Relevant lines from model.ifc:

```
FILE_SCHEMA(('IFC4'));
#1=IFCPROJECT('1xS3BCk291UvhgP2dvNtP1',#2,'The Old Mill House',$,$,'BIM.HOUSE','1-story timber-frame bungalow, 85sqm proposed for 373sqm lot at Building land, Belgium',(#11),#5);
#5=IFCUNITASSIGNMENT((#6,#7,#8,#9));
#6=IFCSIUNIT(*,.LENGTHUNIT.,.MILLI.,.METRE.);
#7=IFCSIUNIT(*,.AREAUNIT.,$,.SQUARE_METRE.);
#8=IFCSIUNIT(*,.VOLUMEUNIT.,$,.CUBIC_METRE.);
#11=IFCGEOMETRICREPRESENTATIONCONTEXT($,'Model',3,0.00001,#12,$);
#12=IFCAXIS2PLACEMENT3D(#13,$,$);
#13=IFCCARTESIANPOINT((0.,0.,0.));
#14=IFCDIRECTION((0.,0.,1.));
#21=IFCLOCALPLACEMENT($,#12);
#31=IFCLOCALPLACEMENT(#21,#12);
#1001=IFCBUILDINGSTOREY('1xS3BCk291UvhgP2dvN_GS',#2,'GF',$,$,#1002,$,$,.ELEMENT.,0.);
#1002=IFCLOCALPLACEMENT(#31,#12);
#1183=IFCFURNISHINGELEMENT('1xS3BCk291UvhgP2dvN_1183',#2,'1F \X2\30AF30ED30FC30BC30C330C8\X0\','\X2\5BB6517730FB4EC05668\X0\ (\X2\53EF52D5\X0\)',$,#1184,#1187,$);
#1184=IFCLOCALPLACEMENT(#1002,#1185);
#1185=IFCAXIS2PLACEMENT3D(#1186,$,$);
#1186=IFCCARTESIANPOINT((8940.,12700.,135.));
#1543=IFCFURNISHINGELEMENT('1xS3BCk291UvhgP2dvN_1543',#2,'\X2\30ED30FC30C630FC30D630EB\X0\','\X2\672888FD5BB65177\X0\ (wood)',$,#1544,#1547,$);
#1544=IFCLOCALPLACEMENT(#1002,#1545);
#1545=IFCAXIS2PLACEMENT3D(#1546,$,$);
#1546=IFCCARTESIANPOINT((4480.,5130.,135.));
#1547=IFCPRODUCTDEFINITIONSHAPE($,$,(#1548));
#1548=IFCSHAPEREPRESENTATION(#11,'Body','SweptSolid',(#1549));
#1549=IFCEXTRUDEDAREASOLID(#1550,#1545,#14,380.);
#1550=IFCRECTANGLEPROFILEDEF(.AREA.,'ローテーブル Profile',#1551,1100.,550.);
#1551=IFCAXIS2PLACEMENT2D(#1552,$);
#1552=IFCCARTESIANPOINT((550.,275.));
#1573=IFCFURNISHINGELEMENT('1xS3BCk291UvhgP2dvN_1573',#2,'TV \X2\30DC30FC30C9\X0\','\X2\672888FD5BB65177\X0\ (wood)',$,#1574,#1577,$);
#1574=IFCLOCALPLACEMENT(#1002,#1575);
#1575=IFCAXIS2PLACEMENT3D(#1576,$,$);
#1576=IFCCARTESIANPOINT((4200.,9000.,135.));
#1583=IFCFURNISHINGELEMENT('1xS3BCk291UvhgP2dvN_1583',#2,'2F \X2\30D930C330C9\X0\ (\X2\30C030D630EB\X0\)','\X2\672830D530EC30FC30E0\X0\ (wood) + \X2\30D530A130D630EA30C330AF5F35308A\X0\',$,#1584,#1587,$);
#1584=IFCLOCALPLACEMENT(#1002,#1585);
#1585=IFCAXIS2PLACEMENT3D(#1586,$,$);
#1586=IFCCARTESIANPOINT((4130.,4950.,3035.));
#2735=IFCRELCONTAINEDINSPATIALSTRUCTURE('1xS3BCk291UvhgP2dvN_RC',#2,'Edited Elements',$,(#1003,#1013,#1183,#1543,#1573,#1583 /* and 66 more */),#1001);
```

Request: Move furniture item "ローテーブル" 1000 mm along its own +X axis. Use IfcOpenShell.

```python
import ifcopenshell
import ifcopenshell.api.geometry
import ifcopenshell.util.placement

model = ifcopenshell.open("model.ifc")

item = model.by_id(1543)
matrix = ifcopenshell.util.placement.get_local_placement(item.ObjectPlacement)
matrix[:3, 3] += matrix[:3, 0] * 1000.0
ifcopenshell.api.geometry.edit_object_placement(model, product=item, matrix=matrix, is_si=False)

print(ifcopenshell.util.placement.get_local_placement(item.ObjectPlacement).round(3) + 0.0)

model.write("model_updated.ifc")
```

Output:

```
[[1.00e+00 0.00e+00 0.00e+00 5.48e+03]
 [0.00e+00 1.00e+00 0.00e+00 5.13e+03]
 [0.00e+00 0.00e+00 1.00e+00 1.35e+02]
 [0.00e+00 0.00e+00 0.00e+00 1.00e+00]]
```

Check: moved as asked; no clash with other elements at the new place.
